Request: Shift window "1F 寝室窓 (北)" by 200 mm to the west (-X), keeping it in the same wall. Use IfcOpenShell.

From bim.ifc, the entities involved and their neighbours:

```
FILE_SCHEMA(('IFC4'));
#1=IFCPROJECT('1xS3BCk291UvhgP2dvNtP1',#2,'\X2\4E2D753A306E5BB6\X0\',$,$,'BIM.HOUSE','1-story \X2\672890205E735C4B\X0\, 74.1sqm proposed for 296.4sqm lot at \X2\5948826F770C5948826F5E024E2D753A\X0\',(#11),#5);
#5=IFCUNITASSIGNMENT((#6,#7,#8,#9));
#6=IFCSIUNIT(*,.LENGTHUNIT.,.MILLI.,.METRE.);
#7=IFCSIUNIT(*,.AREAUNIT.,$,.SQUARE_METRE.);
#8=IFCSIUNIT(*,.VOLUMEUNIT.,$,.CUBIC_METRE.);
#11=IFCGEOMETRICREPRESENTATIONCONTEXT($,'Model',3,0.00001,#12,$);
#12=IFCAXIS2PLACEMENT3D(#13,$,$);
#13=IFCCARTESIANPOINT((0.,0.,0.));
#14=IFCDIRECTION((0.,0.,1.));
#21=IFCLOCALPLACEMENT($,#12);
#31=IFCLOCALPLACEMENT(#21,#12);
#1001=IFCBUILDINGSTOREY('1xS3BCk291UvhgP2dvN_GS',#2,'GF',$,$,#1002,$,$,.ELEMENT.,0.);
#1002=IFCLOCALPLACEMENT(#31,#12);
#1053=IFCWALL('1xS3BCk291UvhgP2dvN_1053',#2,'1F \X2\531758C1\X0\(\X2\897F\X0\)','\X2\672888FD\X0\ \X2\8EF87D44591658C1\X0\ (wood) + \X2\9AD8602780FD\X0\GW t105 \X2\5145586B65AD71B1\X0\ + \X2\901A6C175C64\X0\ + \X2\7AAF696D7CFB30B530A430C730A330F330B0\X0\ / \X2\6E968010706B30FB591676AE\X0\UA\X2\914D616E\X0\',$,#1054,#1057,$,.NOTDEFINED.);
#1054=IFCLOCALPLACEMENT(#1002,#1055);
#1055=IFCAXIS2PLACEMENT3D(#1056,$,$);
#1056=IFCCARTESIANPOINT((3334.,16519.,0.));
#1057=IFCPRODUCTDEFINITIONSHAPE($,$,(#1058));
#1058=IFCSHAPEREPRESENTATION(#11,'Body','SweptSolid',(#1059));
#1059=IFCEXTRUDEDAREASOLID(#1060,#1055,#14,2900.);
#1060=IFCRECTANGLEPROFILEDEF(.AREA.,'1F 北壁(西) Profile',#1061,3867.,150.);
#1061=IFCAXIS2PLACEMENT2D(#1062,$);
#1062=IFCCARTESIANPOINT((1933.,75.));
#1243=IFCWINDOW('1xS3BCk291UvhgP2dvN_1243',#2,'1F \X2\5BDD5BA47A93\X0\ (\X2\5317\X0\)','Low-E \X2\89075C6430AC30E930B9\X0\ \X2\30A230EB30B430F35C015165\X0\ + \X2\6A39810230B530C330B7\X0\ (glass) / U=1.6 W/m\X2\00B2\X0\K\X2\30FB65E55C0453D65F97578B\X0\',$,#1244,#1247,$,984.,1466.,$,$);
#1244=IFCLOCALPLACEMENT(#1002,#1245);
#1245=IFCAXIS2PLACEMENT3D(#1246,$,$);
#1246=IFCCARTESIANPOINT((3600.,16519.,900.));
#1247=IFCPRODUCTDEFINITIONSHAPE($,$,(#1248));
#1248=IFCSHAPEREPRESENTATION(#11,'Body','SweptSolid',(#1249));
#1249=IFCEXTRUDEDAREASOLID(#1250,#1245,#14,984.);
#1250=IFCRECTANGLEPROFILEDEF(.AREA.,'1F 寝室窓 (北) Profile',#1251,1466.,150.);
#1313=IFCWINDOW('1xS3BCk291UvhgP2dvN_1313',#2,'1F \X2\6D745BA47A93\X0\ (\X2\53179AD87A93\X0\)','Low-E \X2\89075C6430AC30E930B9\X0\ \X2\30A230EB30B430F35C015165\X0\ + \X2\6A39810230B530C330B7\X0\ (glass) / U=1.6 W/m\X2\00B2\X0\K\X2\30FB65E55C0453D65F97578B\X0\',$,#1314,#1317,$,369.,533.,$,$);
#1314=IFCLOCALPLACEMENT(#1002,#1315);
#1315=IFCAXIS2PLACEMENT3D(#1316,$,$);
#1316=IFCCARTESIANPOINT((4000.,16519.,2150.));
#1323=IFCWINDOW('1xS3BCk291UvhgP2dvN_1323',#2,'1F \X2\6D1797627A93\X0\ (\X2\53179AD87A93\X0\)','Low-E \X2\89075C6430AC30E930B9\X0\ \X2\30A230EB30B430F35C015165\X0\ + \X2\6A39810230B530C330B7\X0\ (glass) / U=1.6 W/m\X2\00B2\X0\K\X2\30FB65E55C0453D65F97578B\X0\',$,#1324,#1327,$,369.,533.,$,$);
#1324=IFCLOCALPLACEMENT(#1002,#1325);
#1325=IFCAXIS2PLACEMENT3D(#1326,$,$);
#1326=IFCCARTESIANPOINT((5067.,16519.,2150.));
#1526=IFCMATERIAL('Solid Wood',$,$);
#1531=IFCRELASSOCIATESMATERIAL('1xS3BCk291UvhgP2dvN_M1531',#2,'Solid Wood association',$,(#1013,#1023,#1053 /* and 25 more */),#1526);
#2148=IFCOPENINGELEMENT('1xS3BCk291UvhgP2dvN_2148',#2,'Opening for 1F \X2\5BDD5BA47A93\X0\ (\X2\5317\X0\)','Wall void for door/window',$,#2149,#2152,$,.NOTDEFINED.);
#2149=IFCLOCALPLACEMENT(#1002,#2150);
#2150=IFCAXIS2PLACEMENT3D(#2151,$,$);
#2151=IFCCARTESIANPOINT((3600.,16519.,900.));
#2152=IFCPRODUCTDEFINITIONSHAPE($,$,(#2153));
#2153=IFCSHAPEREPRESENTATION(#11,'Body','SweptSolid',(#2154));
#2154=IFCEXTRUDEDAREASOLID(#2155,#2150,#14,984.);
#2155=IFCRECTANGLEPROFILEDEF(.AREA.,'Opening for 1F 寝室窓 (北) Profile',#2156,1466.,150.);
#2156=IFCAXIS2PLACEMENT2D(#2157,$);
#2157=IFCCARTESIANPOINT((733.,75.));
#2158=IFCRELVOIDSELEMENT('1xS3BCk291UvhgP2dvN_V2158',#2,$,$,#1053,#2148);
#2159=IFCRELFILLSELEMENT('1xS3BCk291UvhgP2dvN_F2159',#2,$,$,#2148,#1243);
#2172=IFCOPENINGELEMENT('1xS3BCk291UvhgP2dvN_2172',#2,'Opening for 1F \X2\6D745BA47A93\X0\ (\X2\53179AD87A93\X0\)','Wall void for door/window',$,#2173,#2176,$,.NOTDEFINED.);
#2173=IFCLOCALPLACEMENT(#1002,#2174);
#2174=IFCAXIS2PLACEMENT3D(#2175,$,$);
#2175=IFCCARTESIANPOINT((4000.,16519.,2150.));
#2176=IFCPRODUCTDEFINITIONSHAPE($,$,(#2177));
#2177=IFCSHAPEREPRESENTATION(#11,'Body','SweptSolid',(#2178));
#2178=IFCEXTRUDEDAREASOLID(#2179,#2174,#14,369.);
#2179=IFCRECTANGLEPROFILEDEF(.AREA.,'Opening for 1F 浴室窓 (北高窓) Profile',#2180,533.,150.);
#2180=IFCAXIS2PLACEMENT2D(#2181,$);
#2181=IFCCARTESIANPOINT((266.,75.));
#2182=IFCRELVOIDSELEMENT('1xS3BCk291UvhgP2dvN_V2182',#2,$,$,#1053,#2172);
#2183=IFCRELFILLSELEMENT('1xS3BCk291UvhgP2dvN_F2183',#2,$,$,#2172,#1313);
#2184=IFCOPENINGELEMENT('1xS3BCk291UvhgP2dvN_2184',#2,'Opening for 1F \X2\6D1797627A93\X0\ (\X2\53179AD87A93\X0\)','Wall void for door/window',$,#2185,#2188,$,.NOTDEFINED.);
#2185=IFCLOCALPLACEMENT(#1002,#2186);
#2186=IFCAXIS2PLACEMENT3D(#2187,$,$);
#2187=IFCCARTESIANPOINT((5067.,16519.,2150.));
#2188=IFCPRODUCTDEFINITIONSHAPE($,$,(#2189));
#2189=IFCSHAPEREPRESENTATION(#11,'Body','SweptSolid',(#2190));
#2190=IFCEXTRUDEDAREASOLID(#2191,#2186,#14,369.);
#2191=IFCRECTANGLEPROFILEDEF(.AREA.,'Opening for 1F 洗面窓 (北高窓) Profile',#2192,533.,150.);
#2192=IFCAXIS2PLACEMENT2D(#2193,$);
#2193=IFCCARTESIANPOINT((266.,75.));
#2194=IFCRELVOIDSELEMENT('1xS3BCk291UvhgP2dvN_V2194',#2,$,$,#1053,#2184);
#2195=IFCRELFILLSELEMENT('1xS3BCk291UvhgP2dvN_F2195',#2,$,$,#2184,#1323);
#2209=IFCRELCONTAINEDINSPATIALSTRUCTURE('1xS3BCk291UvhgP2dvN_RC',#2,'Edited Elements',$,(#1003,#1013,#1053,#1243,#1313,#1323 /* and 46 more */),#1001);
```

```python
import ifcopenshell
import ifcopenshell.api.geometry
import ifcopenshell.util.placement

model = ifcopenshell.open("bim.ifc")

window = model.by_id(1243)
opening = window.FillsVoids[0].RelatingOpeningElement
wall = opening.VoidsElements[0].RelatingBuildingElement

wall_matrix = ifcopenshell.util.placement.get_local_placement(wall.ObjectPlacement)
shift = wall_matrix[:3, 0] * -200.0
before = ifcopenshell.util.placement.get_local_placement(window.ObjectPlacement)[:3, 3].copy()

# The window is not placed relative to its opening, so move both.
for product in (opening, window):
    matrix = ifcopenshell.util.placement.get_local_placement(product.ObjectPlacement)
    matrix[:3, 3] += shift
    ifcopenshell.api.geometry.edit_object_placement(model, product=product, matrix=matrix, is_si=False)

after = ifcopenshell.util.placement.get_local_placement(window.ObjectPlacement)[:3, 3]
print("window moved by", (after - before).round(3) + 0.0)

model.write("bim_updated.ifc")
```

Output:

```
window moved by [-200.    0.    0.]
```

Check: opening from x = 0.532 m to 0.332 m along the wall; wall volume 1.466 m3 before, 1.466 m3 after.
